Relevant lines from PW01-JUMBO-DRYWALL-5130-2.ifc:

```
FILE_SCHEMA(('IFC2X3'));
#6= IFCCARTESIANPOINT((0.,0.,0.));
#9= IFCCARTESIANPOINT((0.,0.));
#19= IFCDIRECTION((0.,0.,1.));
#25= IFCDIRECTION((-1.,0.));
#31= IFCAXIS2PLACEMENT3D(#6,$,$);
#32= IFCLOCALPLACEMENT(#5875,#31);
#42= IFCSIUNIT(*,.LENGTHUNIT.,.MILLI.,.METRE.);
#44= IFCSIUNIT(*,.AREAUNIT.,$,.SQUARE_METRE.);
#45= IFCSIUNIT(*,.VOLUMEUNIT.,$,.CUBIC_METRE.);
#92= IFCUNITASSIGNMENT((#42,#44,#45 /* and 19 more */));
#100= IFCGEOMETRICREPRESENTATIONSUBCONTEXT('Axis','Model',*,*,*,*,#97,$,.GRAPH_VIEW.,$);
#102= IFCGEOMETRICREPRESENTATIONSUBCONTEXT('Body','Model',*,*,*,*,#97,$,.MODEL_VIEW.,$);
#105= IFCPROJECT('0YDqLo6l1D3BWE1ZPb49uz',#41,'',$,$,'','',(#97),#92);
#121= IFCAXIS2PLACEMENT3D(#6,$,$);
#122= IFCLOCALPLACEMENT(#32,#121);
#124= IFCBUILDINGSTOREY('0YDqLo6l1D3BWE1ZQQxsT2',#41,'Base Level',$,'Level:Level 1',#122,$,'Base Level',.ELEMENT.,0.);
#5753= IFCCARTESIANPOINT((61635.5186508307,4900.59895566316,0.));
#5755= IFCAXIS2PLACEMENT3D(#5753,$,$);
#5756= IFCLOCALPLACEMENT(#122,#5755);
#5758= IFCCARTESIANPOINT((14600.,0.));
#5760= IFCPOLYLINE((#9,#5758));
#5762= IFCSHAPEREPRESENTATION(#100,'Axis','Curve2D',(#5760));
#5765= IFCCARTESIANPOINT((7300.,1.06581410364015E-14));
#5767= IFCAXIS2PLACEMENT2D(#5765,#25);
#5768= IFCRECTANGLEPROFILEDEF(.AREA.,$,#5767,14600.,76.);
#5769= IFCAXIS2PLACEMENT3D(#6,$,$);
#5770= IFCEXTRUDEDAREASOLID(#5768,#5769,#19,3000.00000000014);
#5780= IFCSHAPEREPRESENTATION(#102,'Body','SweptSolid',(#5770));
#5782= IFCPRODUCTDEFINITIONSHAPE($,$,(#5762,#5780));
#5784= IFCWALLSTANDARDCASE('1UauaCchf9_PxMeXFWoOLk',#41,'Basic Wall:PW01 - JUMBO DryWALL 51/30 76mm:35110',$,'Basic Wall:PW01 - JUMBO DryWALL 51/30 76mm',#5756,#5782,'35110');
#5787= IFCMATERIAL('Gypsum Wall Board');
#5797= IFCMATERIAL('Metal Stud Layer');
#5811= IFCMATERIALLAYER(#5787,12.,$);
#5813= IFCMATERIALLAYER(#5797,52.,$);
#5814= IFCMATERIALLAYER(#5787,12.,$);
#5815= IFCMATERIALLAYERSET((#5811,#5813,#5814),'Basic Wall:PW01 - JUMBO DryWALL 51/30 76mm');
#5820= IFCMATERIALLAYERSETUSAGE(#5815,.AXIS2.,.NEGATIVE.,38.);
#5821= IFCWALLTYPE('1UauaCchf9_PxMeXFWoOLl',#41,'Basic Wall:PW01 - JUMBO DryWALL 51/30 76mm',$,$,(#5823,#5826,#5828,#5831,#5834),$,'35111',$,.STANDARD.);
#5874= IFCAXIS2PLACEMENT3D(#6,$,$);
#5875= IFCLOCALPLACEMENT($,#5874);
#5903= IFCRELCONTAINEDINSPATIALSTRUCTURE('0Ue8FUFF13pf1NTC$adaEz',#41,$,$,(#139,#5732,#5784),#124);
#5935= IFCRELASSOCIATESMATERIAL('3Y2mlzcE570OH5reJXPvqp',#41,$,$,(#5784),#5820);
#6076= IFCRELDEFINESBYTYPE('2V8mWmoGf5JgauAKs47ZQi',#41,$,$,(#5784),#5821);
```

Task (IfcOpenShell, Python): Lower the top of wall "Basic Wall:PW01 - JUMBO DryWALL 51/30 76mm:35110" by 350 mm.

```python
import ifcopenshell
import ifcopenshell.geom
import ifcopenshell.util.representation
import ifcopenshell.util.shape

model = ifcopenshell.open("PW01-JUMBO-DRYWALL-5130-2.ifc")
settings = ifcopenshell.geom.settings()


def volume(element):
    """Net volume in cubic metres, openings subtracted."""
    shape = ifcopenshell.geom.create_shape(settings, element)
    return ifcopenshell.util.shape.get_volume(shape.geometry)


wall = model.by_id(5784)
before = volume(wall)

body = ifcopenshell.util.representation.get_representation(wall, "Model", "Body")
solid = body.Items[0]
old_height = solid.Depth
solid.Depth -= 350.0
after = volume(wall)

print(f"height {old_height:g} -> {solid.Depth:g}, volume {before:.3f} -> {after:.3f} m3")

model.write("PW01-JUMBO-DRYWALL-5130-2_rev.ifc")
```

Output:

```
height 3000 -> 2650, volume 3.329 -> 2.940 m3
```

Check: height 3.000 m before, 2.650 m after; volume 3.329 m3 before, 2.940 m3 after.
